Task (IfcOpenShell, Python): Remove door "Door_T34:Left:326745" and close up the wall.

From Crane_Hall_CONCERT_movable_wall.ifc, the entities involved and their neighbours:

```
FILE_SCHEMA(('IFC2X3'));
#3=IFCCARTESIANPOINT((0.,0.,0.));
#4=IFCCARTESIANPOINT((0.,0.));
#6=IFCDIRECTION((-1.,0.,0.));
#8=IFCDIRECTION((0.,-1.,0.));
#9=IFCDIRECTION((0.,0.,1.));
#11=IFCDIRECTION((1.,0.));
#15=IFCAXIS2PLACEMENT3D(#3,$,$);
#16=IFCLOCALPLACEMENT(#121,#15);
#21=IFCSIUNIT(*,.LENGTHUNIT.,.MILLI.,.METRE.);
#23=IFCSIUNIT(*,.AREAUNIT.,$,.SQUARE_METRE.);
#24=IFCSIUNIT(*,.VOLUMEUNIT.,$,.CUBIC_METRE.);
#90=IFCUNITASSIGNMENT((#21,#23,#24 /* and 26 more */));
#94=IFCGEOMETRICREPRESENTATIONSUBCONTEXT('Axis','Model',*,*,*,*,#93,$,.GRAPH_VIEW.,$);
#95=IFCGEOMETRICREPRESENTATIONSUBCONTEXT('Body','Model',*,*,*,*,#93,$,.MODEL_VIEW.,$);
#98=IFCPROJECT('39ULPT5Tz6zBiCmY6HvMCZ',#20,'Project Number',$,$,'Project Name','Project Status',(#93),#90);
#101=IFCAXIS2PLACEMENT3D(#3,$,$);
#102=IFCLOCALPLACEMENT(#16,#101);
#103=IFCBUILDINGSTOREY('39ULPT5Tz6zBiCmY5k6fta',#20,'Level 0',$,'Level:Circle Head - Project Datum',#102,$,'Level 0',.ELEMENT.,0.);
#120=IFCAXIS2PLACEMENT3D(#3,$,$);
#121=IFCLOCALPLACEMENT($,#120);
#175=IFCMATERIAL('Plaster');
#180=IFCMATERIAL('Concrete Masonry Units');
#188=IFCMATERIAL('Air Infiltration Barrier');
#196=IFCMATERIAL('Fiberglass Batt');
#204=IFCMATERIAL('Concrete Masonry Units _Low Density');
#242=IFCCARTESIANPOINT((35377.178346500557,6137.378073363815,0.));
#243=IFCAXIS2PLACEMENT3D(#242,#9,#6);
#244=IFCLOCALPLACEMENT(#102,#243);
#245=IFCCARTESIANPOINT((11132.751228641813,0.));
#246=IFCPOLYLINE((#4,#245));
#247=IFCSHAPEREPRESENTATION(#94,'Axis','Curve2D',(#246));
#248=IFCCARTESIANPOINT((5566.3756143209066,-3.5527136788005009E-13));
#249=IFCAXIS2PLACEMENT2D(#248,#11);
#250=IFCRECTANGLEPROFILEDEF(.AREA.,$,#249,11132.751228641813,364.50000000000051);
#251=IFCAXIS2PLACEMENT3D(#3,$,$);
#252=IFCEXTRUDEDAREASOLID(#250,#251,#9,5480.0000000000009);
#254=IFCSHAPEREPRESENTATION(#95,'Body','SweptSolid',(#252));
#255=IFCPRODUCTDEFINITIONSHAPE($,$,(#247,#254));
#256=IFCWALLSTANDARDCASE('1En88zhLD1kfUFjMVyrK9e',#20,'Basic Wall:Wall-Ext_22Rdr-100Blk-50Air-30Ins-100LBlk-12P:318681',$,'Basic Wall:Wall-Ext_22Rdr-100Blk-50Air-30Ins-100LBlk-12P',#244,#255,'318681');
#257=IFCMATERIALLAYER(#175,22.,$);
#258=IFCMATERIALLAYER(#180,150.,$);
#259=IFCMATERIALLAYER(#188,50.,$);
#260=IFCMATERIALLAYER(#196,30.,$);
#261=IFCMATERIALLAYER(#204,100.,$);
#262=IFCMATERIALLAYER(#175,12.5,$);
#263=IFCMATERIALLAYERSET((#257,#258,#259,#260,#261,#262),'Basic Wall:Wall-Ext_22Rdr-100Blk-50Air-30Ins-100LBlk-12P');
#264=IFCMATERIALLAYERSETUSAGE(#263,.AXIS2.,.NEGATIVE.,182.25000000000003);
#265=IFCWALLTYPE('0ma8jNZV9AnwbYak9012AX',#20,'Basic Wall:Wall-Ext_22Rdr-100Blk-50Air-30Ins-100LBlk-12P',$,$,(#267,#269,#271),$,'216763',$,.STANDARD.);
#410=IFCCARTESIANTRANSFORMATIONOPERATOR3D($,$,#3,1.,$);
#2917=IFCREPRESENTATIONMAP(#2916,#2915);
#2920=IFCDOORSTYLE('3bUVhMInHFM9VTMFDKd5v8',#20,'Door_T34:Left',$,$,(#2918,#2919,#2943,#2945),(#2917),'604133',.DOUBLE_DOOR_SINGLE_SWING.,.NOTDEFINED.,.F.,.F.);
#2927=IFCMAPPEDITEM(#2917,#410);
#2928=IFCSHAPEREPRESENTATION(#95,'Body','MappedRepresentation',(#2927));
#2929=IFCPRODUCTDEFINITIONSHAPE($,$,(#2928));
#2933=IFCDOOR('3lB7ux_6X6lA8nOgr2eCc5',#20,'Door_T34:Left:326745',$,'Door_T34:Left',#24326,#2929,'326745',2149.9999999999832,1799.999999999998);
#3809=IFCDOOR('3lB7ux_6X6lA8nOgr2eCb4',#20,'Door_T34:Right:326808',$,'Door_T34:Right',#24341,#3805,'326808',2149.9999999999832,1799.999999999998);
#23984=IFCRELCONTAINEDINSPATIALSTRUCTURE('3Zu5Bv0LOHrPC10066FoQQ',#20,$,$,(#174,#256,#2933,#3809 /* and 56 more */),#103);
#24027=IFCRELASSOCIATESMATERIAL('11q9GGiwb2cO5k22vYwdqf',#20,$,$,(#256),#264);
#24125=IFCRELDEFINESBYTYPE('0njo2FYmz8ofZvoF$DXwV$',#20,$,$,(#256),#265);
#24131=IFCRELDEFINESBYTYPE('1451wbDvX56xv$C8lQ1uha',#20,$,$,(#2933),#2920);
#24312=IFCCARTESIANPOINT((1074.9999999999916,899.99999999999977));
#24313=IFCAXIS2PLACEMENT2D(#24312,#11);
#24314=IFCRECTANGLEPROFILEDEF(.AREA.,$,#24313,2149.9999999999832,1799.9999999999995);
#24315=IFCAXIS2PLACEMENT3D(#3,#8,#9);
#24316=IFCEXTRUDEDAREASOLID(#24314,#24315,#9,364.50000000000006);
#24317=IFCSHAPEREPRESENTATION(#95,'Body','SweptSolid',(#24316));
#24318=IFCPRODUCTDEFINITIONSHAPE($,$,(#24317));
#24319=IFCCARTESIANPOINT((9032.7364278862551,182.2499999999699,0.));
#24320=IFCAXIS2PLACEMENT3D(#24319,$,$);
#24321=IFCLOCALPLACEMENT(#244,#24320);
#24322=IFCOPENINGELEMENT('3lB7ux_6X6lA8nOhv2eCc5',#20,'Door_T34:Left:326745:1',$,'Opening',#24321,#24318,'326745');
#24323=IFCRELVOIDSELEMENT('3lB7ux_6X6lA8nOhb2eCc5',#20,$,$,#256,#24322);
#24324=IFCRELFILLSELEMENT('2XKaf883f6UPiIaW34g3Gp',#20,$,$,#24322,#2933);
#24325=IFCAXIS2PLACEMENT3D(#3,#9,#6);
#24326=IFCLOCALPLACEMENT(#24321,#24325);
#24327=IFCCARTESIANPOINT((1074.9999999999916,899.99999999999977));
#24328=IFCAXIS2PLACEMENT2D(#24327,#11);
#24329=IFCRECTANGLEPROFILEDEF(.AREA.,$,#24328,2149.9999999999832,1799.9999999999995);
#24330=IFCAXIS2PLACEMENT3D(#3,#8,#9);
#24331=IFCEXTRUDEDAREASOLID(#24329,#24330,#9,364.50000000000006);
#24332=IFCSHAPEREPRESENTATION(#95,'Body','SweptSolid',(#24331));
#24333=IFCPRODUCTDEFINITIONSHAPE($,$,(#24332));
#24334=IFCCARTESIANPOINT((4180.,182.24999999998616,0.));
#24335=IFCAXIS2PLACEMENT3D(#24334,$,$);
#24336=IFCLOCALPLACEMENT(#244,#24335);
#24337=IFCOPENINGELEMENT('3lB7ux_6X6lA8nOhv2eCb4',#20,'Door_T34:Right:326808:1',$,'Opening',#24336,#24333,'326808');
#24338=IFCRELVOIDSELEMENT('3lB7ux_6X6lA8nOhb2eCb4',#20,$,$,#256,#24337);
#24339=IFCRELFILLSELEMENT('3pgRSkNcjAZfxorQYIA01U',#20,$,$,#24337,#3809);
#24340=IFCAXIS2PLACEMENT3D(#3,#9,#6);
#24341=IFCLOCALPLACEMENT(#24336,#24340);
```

```python
import ifcopenshell
import ifcopenshell.api.feature
import ifcopenshell.api.root
import ifcopenshell.geom
import ifcopenshell.util.shape

model = ifcopenshell.open("Crane_Hall_CONCERT_movable_wall.ifc")
settings = ifcopenshell.geom.settings()


def volume(element):
    """Net volume in cubic metres, openings subtracted."""
    shape = ifcopenshell.geom.create_shape(settings, element)
    return ifcopenshell.util.shape.get_volume(shape.geometry)


door = model.by_guid("3lB7ux_6X6lA8nOgr2eCc5")
opening = door.FillsVoids[0].RelatingOpeningElement
wall = opening.VoidsElements[0].RelatingBuildingElement
before = volume(wall)

ifcopenshell.api.root.remove_product(model, product=door)
ifcopenshell.api.feature.remove_feature(model, feature=opening)

after = volume(wall)

print(f"wall volume {before:.3f} -> {after:.3f} m3")

model.write("Crane_Hall_CONCERT_movable_wall-out.ifc")
```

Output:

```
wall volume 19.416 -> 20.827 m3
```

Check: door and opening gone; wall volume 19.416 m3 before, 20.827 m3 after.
